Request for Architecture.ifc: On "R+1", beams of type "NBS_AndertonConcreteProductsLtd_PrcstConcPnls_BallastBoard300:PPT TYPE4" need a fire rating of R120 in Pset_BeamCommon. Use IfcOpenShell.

First a look at what the model holds.

```python
import ifcopenshell
import ifcopenshell.util.element

model = ifcopenshell.open("Architecture.ifc")
print(model.schema)
storey = next(s for s in model.by_type("IfcBuildingStorey") if s.Name == "R+1")
beams = [e for e in ifcopenshell.util.element.get_decomposition(storey) if e.is_a("IfcBeam")]
seen = {}
for e in beams:
    element_type = ifcopenshell.util.element.get_type(e)
    key = (element_type.Name if element_type != e and element_type else None, ifcopenshell.util.element.get_pset(e, "Pset_BeamCommon", "FireRating"))
    seen[key] = seen.get(key, 0) + 1
for (name, value), count in sorted(seen.items(), key=str):
    print(count, "x", name, "|", value)
```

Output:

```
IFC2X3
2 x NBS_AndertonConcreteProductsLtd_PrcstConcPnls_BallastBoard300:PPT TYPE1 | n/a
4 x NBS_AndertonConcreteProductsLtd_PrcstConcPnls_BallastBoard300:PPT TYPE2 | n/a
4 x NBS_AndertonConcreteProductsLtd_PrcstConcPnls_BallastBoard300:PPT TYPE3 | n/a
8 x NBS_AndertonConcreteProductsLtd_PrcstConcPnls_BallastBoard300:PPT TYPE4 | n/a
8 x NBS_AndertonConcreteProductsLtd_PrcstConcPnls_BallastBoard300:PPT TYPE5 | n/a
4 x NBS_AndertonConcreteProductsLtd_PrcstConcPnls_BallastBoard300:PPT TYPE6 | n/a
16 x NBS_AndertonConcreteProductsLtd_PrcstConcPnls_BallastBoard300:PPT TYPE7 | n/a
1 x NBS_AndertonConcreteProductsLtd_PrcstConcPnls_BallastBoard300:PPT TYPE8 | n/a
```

```python
import ifcopenshell
import ifcopenshell.api.pset
import ifcopenshell.util.element

model = ifcopenshell.open("Architecture.ifc")

storey = next(s for s in model.by_type("IfcBuildingStorey") if s.Name == "R+1")
beams = [e for e in ifcopenshell.util.element.get_decomposition(storey) if e.is_a("IfcBeam")]

count = 0
for e in beams:
    element_type = ifcopenshell.util.element.get_type(e)
    if element_type in (None, e) or element_type.Name != "NBS_AndertonConcreteProductsLtd_PrcstConcPnls_BallastBoard300:PPT TYPE4":
        continue
    # add_pset returns the element's existing set when there is one.
    pset = ifcopenshell.api.pset.add_pset(model, product=e, name="Pset_BeamCommon")
    ifcopenshell.api.pset.edit_pset(model, pset=pset, properties={"FireRating": "R120"})
    count += 1

print(count, "beams updated")

model.write("Architecture_v2.ifc")
```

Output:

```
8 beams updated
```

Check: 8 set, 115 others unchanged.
